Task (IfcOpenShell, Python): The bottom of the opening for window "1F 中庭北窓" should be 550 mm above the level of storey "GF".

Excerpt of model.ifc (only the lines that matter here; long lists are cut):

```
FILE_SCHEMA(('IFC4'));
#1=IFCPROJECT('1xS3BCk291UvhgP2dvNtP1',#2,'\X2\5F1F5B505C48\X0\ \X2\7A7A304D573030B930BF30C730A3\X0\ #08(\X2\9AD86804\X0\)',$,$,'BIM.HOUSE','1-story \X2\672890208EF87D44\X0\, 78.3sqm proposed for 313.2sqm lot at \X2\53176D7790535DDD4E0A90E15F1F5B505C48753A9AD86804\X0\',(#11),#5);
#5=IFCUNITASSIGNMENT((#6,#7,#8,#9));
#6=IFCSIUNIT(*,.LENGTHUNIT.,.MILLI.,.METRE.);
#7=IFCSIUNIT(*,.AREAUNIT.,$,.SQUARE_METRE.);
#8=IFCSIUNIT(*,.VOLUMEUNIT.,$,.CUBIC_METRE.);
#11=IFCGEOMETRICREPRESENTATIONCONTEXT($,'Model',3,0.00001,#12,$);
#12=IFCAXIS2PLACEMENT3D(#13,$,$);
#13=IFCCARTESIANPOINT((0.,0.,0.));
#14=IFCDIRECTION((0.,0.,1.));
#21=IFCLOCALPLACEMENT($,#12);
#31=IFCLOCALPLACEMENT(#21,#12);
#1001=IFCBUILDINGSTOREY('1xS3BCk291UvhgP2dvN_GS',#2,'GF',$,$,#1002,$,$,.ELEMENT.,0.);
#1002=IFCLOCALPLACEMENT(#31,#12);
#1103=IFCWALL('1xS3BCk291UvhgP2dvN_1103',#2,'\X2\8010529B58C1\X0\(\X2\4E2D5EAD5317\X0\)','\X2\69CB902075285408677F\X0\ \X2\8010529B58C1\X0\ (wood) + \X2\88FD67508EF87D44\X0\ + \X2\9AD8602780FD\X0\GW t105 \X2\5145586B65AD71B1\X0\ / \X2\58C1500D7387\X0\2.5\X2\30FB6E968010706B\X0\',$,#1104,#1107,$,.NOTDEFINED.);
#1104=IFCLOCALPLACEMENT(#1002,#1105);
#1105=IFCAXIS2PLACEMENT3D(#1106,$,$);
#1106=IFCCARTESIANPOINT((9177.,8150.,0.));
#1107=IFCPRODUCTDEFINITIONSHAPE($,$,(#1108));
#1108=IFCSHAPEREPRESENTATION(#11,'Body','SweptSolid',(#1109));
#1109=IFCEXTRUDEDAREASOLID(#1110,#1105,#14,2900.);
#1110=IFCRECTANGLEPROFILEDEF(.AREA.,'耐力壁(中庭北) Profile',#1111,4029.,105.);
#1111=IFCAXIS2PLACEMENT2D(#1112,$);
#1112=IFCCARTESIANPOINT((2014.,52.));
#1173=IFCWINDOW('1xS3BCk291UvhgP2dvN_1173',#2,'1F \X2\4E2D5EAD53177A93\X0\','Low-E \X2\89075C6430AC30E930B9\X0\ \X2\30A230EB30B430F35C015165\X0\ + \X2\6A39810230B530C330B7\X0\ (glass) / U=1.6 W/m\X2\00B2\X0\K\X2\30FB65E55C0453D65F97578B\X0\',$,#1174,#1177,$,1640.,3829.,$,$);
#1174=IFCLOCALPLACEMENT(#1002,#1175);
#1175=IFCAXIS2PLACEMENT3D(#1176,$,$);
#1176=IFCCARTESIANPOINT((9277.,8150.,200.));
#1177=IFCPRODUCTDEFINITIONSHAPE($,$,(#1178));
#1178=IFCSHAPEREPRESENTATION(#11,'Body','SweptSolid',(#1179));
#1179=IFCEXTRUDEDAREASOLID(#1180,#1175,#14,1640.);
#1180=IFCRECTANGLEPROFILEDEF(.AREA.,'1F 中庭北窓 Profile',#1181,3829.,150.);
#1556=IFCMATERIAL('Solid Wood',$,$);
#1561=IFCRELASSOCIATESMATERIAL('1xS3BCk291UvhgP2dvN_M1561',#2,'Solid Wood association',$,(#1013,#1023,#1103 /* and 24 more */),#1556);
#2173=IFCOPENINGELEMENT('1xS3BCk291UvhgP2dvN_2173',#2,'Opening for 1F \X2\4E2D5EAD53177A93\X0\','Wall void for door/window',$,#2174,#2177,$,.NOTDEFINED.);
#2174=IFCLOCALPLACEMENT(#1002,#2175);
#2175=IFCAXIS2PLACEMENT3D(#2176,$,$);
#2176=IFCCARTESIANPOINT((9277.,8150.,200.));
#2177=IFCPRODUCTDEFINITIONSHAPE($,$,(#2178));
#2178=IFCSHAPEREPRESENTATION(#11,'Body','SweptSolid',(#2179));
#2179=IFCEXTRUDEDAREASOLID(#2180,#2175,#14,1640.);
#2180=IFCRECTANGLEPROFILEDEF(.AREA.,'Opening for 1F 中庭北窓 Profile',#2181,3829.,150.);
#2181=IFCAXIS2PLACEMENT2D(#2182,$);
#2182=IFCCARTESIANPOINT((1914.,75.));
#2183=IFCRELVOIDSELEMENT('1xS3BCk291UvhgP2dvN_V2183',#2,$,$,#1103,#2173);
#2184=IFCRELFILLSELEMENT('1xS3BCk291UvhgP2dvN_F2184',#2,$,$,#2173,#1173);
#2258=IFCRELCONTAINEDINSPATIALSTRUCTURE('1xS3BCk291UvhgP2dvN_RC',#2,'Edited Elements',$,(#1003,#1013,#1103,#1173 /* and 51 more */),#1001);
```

```python
import numpy as np
import ifcopenshell
import ifcopenshell.api.geometry
import ifcopenshell.geom
import ifcopenshell.util.element
import ifcopenshell.util.placement
import ifcopenshell.util.shape
import ifcopenshell.util.unit

model = ifcopenshell.open("model.ifc")
unit_scale = ifcopenshell.util.unit.calculate_unit_scale(model)

window = model.by_guid("1xS3BCk291UvhgP2dvN_1173")
opening = window.FillsVoids[0].RelatingOpeningElement
storey = ifcopenshell.util.element.get_container(window, ifc_class="IfcBuildingStorey")
level = ifcopenshell.util.placement.get_local_placement(storey.ObjectPlacement)[2, 3]

# The opening's origin need not be at the sill, so measure its lowest point.
shape = ifcopenshell.geom.create_shape(ifcopenshell.geom.settings(), opening)
bottom = ifcopenshell.util.shape.get_shape_bottom_elevation(shape, shape.geometry) / unit_scale
dz = level + 0.55 / unit_scale - bottom

shift = np.array([0.0, 0.0, dz])
# The window is not placed relative to its opening, so move both.
for product in (opening, window):
    matrix = ifcopenshell.util.placement.get_local_placement(product.ObjectPlacement)
    matrix[:3, 3] += shift
    ifcopenshell.api.geometry.edit_object_placement(model, product=product, matrix=matrix, is_si=False)

print(f"moved by {dz * unit_scale:+.3f} m")

model.write("model_v2.ifc")
```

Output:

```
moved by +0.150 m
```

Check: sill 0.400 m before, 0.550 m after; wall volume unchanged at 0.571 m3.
